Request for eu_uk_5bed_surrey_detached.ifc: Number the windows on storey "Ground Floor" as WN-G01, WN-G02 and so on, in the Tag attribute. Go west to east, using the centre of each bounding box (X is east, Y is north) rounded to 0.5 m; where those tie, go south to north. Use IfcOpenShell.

First a look at what the model holds.

```python
import ifcopenshell
import ifcopenshell.util.element
import ifcopenshell.util.placement

model = ifcopenshell.open("eu_uk_5bed_surrey_detached.ifc")
print(model.schema)
storey = next(s for s in model.by_type("IfcBuildingStorey") if s.Name == "Ground Floor")
windows = [e for e in ifcopenshell.util.element.get_decomposition(storey) if e.is_a("IfcWindow")]
for e in sorted(windows, key=lambda e: e.id()):
    origin = ifcopenshell.util.placement.get_local_placement(e.ObjectPlacement)[:3, 3]
    print(e.id(), e.Tag, e.Name, origin.round(2) + 0.0, sep=" | ")
```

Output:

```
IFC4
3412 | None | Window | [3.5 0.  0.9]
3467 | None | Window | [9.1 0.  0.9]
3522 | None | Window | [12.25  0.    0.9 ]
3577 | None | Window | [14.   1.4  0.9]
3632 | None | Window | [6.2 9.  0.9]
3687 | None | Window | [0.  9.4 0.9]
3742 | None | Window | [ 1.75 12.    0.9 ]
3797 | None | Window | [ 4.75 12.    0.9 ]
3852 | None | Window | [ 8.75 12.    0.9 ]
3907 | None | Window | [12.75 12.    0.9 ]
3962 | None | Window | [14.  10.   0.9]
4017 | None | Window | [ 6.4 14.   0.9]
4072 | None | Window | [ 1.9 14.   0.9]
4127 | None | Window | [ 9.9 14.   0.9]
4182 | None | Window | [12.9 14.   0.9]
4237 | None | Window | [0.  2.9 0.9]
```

```python
import ifcopenshell
import ifcopenshell.geom
import ifcopenshell.util.element
import ifcopenshell.util.shape

model = ifcopenshell.open("eu_uk_5bed_surrey_detached.ifc")
settings = ifcopenshell.geom.settings()
settings.set("use-world-coords", True)


def centre(element):
    shape = ifcopenshell.geom.create_shape(settings, element)
    return ifcopenshell.util.shape.get_bbox_centroid(shape.geometry)


storey = next(s for s in model.by_type("IfcBuildingStorey") if s.Name == "Ground Floor")
windows = [e for e in ifcopenshell.util.element.get_decomposition(storey) if e.is_a("IfcWindow")]

# Insertion points can sit at a corner or the storey origin, so sort by the geometry (in metres).
centres = {e: centre(e) for e in windows}
windows.sort(key=lambda e: (round(centres[e][0] / 0.5), centres[e][1]))

for i, e in enumerate(windows, start=1):
    number = f"WN-G{i:02d}"
    e.Tag = number
    print(e.id(), number)

model.write("eu_uk_5bed_surrey_detached_rev.ifc")
```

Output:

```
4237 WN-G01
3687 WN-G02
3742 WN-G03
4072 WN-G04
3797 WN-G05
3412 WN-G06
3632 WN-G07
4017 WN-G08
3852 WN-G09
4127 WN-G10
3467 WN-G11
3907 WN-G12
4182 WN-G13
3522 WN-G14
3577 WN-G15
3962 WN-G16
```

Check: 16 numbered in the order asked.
